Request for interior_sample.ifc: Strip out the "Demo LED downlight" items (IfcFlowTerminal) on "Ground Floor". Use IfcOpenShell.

First a look at what the model holds.

```python
import ifcopenshell
import ifcopenshell.util.element

model = ifcopenshell.open("interior_sample.ifc")
print(model.schema)
storey = next(s for s in model.by_type("IfcBuildingStorey") if s.Name == "Ground Floor")
terminals = [e for e in ifcopenshell.util.element.get_decomposition(storey) if e.is_a("IfcFlowTerminal")]
seen = {}
for e in terminals:
    element_type = ifcopenshell.util.element.get_type(e)
    name = element_type.Name if element_type not in (None, e) else None
    seen[name] = seen.get(name, 0) + 1
for name, count in sorted(seen.items(), key=str):
    print(count, "x", name)
```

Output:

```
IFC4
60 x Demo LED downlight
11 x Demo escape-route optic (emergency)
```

```python
import ifcopenshell
import ifcopenshell.api.root
import ifcopenshell.util.element

model = ifcopenshell.open("interior_sample.ifc")

storey = next(s for s in model.by_type("IfcBuildingStorey") if s.Name == "Ground Floor")
terminals = [e for e in ifcopenshell.util.element.get_decomposition(storey) if e.is_a("IfcFlowTerminal")]
targets = [e for e in terminals if (t := ifcopenshell.util.element.get_type(e)) not in (None, e) and t.Name == "Demo LED downlight"]

for e in targets:
    ifcopenshell.api.root.remove_product(model, product=e)
print(len(targets), "removed")

model.write("interior_sample_edited.ifc")
```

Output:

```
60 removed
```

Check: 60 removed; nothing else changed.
